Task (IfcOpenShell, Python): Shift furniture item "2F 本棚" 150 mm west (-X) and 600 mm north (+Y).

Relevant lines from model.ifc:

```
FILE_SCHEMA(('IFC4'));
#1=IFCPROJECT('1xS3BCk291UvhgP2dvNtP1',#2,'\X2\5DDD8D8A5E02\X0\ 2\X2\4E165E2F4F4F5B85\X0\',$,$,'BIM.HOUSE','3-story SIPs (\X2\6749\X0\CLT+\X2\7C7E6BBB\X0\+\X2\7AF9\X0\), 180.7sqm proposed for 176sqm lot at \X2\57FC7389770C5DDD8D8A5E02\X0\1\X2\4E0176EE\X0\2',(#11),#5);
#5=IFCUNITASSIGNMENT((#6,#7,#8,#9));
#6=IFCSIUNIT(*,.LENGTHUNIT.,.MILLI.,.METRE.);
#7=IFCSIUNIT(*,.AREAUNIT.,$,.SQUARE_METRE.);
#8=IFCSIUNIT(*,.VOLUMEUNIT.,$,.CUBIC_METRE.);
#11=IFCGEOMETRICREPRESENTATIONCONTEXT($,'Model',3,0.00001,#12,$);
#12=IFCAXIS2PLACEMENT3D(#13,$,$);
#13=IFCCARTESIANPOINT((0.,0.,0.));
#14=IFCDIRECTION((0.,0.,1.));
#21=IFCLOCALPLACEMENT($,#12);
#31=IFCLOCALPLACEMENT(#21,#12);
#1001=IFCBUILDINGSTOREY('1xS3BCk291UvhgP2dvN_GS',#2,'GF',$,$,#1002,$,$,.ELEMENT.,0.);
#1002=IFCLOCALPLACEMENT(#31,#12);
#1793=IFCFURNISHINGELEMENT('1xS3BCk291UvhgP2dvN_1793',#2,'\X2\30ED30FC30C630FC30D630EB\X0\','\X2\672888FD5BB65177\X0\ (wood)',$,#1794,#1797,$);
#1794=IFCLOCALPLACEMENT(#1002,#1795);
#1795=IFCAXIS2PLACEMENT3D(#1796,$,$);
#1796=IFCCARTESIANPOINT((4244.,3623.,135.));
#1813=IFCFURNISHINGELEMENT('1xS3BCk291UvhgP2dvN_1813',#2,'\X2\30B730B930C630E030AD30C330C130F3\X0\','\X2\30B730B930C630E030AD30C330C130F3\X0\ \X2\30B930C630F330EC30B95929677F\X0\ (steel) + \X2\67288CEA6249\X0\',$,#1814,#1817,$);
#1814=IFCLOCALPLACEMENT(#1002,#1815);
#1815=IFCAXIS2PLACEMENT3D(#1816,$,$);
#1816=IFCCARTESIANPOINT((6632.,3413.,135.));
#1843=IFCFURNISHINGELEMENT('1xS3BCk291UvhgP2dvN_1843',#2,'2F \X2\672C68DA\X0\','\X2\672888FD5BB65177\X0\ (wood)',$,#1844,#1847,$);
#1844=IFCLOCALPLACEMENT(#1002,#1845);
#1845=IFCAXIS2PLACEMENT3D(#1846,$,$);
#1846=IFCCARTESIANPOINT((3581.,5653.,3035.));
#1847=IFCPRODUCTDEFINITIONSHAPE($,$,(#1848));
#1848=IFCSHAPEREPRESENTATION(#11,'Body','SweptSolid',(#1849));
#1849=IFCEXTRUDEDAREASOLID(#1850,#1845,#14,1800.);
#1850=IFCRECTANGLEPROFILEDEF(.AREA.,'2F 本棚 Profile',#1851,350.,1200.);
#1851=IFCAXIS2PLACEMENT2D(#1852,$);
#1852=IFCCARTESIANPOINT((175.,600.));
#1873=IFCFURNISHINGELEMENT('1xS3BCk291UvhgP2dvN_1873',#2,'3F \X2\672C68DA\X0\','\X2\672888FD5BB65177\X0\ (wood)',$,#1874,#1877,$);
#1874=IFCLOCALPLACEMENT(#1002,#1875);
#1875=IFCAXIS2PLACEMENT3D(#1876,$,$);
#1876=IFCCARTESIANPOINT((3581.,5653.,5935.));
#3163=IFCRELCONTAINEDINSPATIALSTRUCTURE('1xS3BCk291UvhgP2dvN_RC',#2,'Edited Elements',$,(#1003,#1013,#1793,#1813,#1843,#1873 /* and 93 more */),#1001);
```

```python
import ifcopenshell
import ifcopenshell.api.geometry
import ifcopenshell.util.placement
import ifcopenshell.util.unit

model = ifcopenshell.open("model.ifc")
unit_scale = ifcopenshell.util.unit.calculate_unit_scale(model)

item = model.by_guid("1xS3BCk291UvhgP2dvN_1843")
matrix = ifcopenshell.util.placement.get_local_placement(item.ObjectPlacement)
matrix[0, 3] -= 0.15 / unit_scale
matrix[1, 3] += 0.6 / unit_scale
ifcopenshell.api.geometry.edit_object_placement(model, product=item, matrix=matrix, is_si=False)

print(ifcopenshell.util.placement.get_local_placement(item.ObjectPlacement).round(3) + 0.0)

model.write("model_updated.ifc")
```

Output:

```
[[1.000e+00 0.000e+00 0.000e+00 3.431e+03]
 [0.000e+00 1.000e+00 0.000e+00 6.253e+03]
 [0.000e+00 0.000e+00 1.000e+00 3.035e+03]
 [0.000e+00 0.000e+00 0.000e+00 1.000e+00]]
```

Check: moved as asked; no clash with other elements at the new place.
